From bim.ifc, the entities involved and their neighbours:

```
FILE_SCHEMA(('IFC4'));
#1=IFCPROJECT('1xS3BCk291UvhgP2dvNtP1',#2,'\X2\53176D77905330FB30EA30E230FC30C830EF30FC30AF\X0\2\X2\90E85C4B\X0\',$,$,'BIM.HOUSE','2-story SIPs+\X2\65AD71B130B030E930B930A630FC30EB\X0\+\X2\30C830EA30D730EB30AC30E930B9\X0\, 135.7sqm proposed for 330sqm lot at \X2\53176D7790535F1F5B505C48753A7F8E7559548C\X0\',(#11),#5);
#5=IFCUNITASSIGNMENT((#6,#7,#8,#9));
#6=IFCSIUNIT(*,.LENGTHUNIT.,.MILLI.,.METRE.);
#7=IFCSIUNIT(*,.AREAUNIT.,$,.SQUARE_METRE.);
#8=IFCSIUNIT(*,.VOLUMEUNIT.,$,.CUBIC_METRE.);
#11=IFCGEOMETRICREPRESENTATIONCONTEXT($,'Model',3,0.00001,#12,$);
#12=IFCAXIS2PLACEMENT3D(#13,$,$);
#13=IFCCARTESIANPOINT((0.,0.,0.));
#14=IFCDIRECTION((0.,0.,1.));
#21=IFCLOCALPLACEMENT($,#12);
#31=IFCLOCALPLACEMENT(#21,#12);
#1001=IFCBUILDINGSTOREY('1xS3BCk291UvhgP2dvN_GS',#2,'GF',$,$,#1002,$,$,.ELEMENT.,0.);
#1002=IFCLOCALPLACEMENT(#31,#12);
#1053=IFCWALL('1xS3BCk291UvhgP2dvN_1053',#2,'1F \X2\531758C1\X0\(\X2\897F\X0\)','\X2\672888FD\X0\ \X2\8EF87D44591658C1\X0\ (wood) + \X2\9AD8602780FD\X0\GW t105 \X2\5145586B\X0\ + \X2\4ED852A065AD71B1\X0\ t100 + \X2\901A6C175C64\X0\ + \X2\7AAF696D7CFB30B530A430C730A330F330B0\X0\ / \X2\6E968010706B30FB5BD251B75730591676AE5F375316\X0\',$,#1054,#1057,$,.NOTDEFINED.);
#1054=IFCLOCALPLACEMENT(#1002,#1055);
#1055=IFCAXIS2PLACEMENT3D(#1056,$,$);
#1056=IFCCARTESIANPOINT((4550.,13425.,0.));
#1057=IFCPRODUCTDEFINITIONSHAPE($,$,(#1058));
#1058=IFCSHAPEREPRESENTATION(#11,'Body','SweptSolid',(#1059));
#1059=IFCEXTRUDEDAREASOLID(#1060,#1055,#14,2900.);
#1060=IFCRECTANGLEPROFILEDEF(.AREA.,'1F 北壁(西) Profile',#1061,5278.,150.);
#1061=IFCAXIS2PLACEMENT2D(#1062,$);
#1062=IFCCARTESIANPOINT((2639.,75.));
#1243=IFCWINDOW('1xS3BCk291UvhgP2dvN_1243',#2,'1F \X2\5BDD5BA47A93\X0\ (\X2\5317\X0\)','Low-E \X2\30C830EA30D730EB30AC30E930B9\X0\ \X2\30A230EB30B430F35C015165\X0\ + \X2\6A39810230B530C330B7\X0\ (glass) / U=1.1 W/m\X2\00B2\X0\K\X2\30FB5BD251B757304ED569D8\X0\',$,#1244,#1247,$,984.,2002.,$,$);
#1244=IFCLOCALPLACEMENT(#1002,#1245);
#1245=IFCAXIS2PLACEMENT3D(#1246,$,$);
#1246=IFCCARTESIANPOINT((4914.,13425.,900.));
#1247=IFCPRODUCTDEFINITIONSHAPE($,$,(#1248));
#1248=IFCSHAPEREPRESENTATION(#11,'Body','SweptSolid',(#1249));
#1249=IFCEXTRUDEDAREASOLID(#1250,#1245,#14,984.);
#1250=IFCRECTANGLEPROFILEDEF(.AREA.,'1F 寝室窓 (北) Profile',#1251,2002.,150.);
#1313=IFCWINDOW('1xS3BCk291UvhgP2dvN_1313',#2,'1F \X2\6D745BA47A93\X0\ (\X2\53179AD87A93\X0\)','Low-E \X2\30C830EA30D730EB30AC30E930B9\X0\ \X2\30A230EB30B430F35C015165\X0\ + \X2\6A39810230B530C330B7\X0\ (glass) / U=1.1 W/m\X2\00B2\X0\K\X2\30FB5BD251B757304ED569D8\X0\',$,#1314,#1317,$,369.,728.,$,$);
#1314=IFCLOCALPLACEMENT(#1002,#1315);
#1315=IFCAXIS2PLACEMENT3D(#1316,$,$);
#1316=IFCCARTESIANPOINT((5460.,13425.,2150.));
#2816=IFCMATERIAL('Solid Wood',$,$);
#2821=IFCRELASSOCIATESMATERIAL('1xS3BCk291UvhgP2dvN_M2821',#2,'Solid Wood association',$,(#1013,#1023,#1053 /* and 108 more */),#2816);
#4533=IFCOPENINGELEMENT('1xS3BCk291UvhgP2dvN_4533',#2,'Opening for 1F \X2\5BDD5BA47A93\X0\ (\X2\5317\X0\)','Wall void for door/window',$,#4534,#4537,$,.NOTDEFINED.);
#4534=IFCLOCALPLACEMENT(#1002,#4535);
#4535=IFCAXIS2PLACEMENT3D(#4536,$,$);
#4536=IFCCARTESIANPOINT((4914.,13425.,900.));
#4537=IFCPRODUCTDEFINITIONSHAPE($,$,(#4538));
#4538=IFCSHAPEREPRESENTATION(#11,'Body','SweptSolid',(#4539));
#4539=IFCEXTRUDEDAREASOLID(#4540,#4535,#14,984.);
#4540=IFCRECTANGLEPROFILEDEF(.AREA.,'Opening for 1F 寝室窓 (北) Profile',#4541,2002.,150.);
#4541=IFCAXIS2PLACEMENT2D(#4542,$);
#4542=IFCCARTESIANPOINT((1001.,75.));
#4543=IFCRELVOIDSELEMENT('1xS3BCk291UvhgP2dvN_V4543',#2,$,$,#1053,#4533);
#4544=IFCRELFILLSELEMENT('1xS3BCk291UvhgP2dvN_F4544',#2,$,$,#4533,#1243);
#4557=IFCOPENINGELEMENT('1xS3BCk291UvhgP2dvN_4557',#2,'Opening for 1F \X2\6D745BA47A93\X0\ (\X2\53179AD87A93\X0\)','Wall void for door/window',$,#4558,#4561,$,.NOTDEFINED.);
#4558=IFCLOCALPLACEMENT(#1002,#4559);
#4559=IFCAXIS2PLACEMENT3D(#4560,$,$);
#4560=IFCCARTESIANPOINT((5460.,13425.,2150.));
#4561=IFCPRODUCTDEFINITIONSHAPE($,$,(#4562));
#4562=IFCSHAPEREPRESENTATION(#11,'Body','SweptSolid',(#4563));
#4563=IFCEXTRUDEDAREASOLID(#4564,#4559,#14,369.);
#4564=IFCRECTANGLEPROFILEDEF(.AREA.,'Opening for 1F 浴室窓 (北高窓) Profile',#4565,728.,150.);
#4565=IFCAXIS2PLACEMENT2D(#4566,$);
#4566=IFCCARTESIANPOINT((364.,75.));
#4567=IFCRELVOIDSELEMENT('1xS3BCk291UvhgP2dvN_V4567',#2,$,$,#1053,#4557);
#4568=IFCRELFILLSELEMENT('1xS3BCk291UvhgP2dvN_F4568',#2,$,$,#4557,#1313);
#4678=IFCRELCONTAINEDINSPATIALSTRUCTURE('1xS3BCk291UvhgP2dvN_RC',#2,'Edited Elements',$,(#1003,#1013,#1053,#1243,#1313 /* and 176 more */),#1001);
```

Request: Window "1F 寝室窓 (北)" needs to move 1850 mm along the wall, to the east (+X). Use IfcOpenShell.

```python
import ifcopenshell
import ifcopenshell.api.geometry
import ifcopenshell.util.placement

model = ifcopenshell.open("bim.ifc")

window = model.by_guid("1xS3BCk291UvhgP2dvN_1243")
opening = window.FillsVoids[0].RelatingOpeningElement
wall = opening.VoidsElements[0].RelatingBuildingElement

wall_matrix = ifcopenshell.util.placement.get_local_placement(wall.ObjectPlacement)
shift = wall_matrix[:3, 0] * 1850.0
before = ifcopenshell.util.placement.get_local_placement(window.ObjectPlacement)[:3, 3].copy()

# The window is not placed relative to its opening, so move both.
for product in (opening, window):
    matrix = ifcopenshell.util.placement.get_local_placement(product.ObjectPlacement)
    matrix[:3, 3] += shift
    ifcopenshell.api.geometry.edit_object_placement(model, product=product, matrix=matrix, is_si=False)

after = ifcopenshell.util.placement.get_local_placement(window.ObjectPlacement)[:3, 3]
print("window moved by", (after - before).round(3) + 0.0)

model.write("bim_edited.ifc")
```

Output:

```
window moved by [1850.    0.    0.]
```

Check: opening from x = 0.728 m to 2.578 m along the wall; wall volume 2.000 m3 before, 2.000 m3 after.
